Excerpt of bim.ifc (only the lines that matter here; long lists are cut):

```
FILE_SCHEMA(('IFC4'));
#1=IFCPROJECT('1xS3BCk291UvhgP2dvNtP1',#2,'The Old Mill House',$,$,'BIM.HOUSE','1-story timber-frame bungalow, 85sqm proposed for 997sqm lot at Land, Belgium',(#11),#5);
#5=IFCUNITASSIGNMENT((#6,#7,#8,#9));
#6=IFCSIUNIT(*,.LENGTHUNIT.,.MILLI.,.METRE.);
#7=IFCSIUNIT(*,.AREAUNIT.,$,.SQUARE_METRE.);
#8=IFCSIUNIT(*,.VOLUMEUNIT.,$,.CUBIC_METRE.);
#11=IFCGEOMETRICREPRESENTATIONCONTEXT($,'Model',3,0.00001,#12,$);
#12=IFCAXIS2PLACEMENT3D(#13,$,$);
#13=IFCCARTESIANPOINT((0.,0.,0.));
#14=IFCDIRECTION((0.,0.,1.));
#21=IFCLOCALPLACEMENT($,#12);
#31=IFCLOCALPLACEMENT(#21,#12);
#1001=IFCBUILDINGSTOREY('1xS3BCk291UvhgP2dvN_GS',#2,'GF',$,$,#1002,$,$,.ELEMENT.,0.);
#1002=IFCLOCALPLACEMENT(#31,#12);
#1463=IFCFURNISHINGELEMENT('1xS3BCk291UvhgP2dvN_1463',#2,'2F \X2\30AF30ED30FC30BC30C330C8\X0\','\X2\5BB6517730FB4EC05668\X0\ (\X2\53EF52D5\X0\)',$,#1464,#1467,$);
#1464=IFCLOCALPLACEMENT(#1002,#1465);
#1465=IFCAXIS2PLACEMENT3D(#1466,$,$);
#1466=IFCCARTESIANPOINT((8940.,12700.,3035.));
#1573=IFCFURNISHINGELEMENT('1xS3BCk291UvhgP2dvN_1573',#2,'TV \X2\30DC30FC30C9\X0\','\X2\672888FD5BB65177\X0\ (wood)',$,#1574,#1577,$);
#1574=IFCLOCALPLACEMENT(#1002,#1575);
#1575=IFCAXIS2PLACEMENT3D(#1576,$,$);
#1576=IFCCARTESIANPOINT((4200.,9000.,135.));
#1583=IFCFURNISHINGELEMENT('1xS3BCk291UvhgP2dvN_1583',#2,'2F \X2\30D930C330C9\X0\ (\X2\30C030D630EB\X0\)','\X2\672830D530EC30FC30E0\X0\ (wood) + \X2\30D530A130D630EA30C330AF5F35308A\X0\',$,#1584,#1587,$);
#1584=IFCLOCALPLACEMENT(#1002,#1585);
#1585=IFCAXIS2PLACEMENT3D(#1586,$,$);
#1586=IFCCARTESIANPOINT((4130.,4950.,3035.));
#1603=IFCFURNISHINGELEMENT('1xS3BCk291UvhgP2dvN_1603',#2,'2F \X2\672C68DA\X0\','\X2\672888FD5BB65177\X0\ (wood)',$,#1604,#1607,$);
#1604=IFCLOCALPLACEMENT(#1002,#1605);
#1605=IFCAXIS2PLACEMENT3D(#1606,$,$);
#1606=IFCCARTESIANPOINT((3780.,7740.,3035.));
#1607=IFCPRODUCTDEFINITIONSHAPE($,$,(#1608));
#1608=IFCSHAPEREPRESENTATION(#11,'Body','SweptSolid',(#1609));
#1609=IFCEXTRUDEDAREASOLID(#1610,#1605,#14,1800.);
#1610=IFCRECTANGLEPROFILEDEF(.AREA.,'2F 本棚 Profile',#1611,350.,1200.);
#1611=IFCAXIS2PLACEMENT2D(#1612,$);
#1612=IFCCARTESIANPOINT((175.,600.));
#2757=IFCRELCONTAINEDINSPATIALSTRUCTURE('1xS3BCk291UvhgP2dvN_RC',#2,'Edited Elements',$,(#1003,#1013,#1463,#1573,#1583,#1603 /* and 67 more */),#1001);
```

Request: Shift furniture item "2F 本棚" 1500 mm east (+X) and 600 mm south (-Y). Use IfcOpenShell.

```python
import ifcopenshell
import ifcopenshell.api.geometry
import ifcopenshell.util.placement
import ifcopenshell.util.unit

model = ifcopenshell.open("bim.ifc")
unit_scale = ifcopenshell.util.unit.calculate_unit_scale(model)

item = model.by_guid("1xS3BCk291UvhgP2dvN_1603")
matrix = ifcopenshell.util.placement.get_local_placement(item.ObjectPlacement)
matrix[0, 3] += 1.5 / unit_scale
matrix[1, 3] -= 0.6 / unit_scale
ifcopenshell.api.geometry.edit_object_placement(model, product=item, matrix=matrix, is_si=False)

print(ifcopenshell.util.placement.get_local_placement(item.ObjectPlacement).round(3) + 0.0)

model.write("bim-out.ifc")
```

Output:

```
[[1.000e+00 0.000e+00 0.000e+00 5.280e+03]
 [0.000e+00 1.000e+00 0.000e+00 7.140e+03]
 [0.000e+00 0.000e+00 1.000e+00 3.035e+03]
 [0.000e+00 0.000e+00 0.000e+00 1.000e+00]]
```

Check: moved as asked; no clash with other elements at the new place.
